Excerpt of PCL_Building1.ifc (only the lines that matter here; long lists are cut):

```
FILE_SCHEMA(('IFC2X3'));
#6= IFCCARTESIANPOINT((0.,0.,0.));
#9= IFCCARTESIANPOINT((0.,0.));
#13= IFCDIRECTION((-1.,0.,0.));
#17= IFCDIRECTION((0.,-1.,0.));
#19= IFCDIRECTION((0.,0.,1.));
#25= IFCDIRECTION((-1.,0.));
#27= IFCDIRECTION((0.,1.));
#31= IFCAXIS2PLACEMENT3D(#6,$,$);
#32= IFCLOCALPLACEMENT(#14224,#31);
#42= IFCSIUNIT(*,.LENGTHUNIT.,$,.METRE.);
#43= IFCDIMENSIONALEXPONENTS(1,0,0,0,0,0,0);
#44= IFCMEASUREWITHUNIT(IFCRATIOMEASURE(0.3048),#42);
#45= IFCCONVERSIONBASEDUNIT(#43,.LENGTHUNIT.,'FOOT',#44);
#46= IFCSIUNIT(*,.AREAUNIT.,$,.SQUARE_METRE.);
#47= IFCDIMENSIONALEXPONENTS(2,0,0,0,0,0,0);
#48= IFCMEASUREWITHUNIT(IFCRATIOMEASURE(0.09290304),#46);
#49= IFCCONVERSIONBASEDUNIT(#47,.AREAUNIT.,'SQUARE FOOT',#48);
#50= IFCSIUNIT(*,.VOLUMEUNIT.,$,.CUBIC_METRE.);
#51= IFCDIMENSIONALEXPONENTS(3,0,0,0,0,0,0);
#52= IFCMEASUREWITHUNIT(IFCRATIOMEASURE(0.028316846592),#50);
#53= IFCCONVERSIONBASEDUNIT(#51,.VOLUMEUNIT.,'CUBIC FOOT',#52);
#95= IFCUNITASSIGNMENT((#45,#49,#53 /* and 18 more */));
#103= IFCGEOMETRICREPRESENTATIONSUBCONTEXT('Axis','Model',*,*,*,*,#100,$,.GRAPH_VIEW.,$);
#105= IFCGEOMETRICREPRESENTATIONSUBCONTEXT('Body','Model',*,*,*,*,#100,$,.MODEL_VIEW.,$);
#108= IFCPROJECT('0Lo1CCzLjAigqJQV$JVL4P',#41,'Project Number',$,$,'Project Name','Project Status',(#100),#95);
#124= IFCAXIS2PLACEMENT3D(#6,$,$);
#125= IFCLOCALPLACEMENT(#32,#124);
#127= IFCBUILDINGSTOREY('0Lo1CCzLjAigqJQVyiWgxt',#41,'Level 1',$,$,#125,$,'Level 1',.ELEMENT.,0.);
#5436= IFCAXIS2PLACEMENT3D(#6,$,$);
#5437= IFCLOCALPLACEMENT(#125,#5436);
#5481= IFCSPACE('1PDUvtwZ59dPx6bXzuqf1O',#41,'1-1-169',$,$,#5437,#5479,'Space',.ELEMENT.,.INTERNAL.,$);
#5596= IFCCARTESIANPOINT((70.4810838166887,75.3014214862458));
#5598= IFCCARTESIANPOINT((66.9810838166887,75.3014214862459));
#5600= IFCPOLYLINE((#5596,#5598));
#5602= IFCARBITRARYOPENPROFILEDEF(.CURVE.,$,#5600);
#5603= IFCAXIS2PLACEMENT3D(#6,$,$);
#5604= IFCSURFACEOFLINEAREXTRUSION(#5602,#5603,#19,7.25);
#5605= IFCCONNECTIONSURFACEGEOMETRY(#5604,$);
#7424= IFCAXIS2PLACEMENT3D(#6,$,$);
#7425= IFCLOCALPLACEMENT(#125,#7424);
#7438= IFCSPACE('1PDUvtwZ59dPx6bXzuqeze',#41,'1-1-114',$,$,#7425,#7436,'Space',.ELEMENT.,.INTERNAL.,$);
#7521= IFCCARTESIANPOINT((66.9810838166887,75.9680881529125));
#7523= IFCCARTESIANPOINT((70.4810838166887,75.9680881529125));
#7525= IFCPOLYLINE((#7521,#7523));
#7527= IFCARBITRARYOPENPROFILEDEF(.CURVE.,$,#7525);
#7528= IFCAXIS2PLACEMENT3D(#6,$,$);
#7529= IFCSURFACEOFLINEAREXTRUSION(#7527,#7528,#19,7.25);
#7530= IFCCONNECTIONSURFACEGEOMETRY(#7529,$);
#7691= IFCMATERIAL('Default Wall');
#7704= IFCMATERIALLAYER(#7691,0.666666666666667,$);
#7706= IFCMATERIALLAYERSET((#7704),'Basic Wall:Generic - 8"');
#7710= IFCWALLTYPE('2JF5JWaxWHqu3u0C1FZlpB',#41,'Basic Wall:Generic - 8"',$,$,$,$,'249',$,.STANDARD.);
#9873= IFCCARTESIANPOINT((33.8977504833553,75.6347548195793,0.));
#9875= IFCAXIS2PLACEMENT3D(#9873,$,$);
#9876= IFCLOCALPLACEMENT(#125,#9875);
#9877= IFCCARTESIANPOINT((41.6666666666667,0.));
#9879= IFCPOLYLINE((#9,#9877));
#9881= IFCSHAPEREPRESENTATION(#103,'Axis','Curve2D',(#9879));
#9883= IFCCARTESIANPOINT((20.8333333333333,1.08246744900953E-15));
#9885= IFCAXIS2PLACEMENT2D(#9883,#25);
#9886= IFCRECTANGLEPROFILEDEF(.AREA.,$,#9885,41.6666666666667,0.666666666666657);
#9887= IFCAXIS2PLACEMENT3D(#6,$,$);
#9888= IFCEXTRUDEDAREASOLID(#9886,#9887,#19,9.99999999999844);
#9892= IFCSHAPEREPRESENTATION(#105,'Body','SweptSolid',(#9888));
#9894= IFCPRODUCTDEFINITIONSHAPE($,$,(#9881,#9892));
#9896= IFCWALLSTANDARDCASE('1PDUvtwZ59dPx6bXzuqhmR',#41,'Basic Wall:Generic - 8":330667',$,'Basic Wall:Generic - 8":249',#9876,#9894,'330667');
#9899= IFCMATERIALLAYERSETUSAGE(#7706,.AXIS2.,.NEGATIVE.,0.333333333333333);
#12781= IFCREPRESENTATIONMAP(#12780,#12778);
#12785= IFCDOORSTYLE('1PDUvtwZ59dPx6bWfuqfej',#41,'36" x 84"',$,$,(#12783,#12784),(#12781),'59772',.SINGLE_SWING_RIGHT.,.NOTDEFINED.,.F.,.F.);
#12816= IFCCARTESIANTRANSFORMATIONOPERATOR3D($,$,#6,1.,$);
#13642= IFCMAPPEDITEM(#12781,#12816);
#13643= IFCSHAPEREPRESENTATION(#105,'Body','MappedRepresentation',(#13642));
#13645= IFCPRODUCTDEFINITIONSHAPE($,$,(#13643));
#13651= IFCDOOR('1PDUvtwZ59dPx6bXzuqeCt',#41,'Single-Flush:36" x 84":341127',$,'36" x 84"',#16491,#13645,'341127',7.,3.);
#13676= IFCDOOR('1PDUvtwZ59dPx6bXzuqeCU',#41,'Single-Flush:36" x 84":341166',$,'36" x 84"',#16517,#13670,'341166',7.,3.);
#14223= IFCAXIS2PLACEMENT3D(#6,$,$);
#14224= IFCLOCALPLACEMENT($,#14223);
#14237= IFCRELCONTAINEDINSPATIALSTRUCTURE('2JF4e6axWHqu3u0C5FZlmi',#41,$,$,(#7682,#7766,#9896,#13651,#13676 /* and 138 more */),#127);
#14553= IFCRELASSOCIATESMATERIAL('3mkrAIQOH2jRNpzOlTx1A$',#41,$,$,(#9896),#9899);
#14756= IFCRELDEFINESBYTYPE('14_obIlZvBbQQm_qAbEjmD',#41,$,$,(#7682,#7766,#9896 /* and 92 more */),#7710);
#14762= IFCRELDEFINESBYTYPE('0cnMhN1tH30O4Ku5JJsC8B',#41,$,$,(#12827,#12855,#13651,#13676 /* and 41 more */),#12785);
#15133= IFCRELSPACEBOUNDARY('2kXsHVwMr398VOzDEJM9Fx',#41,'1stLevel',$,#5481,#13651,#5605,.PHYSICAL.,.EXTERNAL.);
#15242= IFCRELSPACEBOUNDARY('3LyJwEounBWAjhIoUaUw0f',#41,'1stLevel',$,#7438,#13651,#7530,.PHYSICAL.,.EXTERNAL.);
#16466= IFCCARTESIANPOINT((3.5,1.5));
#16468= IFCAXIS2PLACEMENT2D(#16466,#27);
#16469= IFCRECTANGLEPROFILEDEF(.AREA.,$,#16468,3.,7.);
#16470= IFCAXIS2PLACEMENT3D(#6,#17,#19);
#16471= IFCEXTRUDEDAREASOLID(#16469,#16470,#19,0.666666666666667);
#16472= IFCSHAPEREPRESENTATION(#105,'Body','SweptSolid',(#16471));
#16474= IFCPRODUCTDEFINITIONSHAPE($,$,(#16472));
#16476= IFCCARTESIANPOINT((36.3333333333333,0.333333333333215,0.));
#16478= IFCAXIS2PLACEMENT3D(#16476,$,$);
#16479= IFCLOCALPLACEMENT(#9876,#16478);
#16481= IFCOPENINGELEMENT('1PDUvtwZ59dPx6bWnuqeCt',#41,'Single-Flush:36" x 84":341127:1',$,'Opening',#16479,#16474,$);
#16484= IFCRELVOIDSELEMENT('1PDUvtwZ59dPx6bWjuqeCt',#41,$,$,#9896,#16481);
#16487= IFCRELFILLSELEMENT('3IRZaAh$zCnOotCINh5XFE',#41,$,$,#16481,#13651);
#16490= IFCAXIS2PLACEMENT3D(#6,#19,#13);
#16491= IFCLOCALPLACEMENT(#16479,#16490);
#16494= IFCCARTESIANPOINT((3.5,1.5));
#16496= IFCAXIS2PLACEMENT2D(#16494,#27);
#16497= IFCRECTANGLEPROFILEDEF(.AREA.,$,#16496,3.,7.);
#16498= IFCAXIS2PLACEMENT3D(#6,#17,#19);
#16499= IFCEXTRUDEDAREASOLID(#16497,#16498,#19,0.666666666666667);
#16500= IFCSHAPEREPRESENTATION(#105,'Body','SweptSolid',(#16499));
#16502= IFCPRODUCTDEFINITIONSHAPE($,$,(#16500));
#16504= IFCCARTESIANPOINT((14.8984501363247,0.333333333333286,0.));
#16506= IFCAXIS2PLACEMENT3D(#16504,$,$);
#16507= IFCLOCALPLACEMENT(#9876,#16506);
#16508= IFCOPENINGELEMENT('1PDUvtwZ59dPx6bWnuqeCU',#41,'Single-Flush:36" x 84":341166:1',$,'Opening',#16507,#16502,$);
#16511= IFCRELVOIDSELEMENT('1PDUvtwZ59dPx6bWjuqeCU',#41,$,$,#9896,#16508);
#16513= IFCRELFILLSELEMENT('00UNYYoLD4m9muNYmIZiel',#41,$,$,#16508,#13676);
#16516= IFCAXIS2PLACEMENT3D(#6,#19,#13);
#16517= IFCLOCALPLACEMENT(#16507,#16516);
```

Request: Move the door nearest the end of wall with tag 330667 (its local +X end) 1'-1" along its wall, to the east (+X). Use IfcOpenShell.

```python
import numpy as np
import ifcopenshell
import ifcopenshell.api.geometry
import ifcopenshell.util.placement
import ifcopenshell.util.unit

model = ifcopenshell.open("PCL_Building1.ifc")
unit_scale = ifcopenshell.util.unit.calculate_unit_scale(model)

door = model.by_guid("1PDUvtwZ59dPx6bXzuqeCt")
opening = door.FillsVoids[0].RelatingOpeningElement
wall = opening.VoidsElements[0].RelatingBuildingElement

wall_matrix = ifcopenshell.util.placement.get_local_placement(wall.ObjectPlacement)
shift = wall_matrix[:3, 0] * 13 * 0.0254 / unit_scale
before = ifcopenshell.util.placement.get_local_placement(door.ObjectPlacement)[:3, 3].copy()

# The door is placed relative to its opening, so it follows when the opening moves.
matrix = ifcopenshell.util.placement.get_local_placement(opening.ObjectPlacement)
matrix[:3, 3] += shift
ifcopenshell.api.geometry.edit_object_placement(
    model, product=opening, matrix=matrix, is_si=False, should_transform_children=True
)

# Space boundary surfaces are stored in each space's coordinates; move them too.
for rel in door.ProvidesBoundaries:
    if not rel.ConnectionGeometry:
        continue
    surface = rel.ConnectionGeometry.SurfaceOnRelatingElement
    space_matrix = ifcopenshell.util.placement.get_local_placement(rel.RelatingSpace.ObjectPlacement)
    point = np.array(surface.Position.Location.Coordinates) + space_matrix[:3, :3].T @ shift
    surface.Position = model.createIfcAxis2Placement3D(
        model.createIfcCartesianPoint(point.tolist()), surface.Position.Axis, surface.Position.RefDirection
    )

after = ifcopenshell.util.placement.get_local_placement(door.ObjectPlacement)[:3, 3]
print("door moved by", (after - before).round(3) + 0.0)

model.write("PCL_Building1_v2.ifc")
```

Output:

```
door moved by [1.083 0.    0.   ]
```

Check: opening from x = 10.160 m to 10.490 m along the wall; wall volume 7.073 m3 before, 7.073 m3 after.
